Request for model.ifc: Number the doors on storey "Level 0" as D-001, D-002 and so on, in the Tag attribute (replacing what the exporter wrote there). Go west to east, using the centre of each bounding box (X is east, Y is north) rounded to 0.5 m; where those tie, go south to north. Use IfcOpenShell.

First a look at what the model holds.

```python
import ifcopenshell
import ifcopenshell.util.element
import ifcopenshell.util.placement

model = ifcopenshell.open("model.ifc")
print(model.schema)
storey = next(s for s in model.by_type("IfcBuildingStorey") if s.Name == "Level 0")
doors = [e for e in ifcopenshell.util.element.get_decomposition(storey) if e.is_a("IfcDoor")]
for e in sorted(doors, key=lambda e: e.id()):
    origin = ifcopenshell.util.placement.get_local_placement(e.ObjectPlacement)[:3, 3]
    print(e.id(), e.Tag, e.Name, origin.round(2) + 0.0, sep=" | ")
```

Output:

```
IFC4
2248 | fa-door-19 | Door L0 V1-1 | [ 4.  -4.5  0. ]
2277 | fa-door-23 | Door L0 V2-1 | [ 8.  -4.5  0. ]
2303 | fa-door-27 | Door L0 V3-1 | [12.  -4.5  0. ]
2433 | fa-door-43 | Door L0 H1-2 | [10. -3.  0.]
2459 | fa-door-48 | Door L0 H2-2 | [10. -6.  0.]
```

```python
import ifcopenshell
import ifcopenshell.geom
import ifcopenshell.util.element
import ifcopenshell.util.shape

model = ifcopenshell.open("model.ifc")
settings = ifcopenshell.geom.settings()
settings.set("use-world-coords", True)


def centre(element):
    shape = ifcopenshell.geom.create_shape(settings, element)
    return ifcopenshell.util.shape.get_bbox_centroid(shape.geometry)


storey = next(s for s in model.by_type("IfcBuildingStorey") if s.Name == "Level 0")
doors = [e for e in ifcopenshell.util.element.get_decomposition(storey) if e.is_a("IfcDoor")]

# Insertion points can sit at a corner or the storey origin, so sort by the geometry (in metres).
centres = {e: centre(e) for e in doors}
doors.sort(key=lambda e: (round(centres[e][0] / 0.5), centres[e][1]))

for i, e in enumerate(doors, start=1):
    number = f"D-0{i:02d}"
    e.Tag = number
    print(e.id(), number)

model.write("model_updated.ifc")
```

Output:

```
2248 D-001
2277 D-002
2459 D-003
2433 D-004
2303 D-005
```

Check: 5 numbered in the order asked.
